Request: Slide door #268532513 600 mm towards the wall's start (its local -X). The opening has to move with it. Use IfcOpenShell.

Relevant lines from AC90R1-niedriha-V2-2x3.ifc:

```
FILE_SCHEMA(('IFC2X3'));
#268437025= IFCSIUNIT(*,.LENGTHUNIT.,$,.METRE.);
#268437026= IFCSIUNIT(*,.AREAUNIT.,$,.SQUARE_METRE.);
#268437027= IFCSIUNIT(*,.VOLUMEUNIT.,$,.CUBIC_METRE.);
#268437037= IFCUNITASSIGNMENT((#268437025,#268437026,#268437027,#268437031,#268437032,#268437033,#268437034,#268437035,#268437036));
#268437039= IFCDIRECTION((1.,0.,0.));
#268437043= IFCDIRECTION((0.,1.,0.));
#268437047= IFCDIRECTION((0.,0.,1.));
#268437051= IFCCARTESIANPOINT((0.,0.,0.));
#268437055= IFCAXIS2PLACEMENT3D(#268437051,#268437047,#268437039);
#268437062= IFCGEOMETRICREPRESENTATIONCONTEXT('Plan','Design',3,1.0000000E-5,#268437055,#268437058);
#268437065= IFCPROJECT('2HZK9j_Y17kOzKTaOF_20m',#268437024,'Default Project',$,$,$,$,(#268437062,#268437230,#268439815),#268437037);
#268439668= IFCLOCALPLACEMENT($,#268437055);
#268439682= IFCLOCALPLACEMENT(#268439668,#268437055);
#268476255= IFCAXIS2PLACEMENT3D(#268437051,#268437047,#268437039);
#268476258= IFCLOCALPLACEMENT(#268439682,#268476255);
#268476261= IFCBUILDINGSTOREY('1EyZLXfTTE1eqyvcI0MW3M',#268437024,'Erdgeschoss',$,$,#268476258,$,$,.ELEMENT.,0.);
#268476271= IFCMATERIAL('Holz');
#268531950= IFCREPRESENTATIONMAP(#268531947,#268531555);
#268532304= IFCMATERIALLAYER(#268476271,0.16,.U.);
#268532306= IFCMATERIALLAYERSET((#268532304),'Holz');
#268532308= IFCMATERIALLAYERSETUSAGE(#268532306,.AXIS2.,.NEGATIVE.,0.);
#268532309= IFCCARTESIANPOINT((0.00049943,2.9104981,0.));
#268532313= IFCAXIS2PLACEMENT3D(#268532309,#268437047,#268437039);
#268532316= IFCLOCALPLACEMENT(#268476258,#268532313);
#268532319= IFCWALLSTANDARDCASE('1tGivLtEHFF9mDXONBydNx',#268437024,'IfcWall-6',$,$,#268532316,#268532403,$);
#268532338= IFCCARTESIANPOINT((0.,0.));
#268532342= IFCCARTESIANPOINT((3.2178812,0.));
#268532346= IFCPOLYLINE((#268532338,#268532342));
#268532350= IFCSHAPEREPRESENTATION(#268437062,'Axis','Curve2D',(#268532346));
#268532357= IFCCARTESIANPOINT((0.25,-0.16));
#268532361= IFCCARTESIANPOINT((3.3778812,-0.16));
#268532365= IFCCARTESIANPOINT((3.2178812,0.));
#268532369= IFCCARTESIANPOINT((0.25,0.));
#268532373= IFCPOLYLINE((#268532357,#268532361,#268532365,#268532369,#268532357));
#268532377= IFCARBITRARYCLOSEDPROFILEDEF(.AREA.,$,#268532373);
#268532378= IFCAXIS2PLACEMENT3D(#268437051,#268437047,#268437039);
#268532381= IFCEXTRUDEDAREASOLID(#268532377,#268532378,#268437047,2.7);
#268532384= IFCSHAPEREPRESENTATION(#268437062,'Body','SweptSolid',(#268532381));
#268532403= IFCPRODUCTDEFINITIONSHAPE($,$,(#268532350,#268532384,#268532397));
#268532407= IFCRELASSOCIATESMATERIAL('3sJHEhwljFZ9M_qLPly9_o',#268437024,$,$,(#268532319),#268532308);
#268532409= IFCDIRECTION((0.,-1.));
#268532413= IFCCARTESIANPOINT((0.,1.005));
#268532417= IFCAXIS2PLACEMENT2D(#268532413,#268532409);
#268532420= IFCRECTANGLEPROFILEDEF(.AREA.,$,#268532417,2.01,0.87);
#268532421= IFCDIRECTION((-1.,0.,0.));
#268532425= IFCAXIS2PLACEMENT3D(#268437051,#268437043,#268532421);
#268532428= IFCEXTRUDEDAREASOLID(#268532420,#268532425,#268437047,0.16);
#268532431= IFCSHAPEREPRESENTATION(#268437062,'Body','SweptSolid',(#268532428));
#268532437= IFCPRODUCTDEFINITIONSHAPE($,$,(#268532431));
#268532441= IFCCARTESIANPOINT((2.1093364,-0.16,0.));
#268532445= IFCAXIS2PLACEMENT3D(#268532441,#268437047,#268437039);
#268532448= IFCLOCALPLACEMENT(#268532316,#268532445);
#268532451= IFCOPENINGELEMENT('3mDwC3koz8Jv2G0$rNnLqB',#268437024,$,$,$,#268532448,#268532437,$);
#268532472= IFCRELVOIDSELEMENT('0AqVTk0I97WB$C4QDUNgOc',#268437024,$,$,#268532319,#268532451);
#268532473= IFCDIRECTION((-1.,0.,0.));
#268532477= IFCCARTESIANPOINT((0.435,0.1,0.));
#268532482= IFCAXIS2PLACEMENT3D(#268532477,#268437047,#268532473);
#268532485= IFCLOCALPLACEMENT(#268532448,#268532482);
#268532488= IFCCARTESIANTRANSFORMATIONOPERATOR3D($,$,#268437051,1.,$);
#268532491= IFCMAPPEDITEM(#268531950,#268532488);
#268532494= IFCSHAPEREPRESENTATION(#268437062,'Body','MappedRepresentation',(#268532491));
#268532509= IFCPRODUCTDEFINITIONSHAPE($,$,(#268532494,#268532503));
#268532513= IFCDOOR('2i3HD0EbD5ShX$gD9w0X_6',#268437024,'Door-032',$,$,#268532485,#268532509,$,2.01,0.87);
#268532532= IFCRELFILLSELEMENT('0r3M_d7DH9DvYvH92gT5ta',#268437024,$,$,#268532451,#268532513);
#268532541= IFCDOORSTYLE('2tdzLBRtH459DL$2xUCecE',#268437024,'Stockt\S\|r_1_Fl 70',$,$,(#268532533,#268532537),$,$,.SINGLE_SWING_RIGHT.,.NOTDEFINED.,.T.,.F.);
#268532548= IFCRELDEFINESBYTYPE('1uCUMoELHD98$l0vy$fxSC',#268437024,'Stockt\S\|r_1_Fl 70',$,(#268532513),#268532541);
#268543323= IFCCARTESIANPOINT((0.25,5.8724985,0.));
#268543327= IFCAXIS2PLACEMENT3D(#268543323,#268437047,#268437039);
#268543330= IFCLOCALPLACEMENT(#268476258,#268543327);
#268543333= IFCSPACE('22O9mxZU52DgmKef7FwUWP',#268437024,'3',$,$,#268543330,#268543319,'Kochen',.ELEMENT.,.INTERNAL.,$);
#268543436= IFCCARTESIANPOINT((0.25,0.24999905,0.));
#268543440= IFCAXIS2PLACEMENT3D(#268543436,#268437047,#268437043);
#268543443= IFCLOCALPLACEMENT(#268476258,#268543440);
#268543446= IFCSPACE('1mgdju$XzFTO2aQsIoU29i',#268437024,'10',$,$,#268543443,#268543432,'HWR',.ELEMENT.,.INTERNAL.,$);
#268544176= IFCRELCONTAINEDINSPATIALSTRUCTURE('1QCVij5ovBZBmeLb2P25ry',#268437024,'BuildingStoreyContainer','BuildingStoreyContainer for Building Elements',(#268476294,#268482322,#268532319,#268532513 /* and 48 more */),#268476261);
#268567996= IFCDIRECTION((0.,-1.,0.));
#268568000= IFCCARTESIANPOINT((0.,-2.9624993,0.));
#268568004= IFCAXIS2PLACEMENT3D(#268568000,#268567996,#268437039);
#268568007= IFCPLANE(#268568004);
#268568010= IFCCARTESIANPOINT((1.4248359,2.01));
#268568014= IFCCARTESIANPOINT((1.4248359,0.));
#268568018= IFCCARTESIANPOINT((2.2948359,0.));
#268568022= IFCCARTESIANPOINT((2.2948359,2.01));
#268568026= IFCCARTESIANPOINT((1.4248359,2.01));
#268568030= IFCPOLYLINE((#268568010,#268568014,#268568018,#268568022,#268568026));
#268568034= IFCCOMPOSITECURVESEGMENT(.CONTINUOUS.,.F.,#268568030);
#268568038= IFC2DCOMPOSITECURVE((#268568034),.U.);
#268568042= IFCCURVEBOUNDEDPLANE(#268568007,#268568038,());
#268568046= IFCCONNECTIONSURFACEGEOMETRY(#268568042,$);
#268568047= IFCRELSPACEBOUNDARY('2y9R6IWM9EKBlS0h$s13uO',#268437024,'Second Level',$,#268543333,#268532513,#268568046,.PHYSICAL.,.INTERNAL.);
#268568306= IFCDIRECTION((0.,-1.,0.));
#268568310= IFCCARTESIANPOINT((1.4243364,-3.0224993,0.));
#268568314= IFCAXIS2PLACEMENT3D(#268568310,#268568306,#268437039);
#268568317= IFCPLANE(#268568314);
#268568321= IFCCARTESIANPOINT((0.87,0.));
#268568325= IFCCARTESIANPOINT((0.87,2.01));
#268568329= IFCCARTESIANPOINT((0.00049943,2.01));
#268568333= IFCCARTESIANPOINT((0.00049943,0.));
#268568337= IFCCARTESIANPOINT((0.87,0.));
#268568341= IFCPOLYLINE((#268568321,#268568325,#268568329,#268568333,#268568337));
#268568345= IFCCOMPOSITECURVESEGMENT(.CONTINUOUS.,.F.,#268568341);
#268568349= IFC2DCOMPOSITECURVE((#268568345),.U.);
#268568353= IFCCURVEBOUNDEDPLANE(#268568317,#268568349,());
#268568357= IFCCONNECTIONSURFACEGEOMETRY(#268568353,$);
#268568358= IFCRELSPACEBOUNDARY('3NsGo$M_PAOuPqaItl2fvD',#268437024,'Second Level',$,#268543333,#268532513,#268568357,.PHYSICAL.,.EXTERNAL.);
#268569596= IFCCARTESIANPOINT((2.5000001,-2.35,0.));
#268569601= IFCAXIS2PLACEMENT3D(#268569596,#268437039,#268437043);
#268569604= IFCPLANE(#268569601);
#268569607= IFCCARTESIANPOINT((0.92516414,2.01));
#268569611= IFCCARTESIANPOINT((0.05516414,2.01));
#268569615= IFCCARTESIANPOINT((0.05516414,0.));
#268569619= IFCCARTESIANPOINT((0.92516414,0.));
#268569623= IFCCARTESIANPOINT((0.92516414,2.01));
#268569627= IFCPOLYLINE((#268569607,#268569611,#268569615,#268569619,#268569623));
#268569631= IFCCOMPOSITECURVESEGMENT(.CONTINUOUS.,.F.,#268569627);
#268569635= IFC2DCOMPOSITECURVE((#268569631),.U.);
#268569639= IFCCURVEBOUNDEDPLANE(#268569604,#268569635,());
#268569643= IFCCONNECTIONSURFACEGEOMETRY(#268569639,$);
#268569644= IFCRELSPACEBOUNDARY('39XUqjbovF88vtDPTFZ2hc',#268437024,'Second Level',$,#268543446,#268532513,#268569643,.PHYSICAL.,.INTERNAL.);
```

```python
import numpy as np
import ifcopenshell
import ifcopenshell.api.geometry
import ifcopenshell.util.placement

model = ifcopenshell.open("AC90R1-niedriha-V2-2x3.ifc")

door = model.by_guid("2i3HD0EbD5ShX$gD9w0X_6")
opening = door.FillsVoids[0].RelatingOpeningElement
wall = opening.VoidsElements[0].RelatingBuildingElement

wall_matrix = ifcopenshell.util.placement.get_local_placement(wall.ObjectPlacement)
shift = wall_matrix[:3, 0] * -0.6
before = ifcopenshell.util.placement.get_local_placement(door.ObjectPlacement)[:3, 3].copy()

# The door is placed relative to its opening, so it follows when the opening moves.
matrix = ifcopenshell.util.placement.get_local_placement(opening.ObjectPlacement)
matrix[:3, 3] += shift
ifcopenshell.api.geometry.edit_object_placement(
    model, product=opening, matrix=matrix, is_si=False, should_transform_children=True
)

# Space boundary surfaces are stored in each space's coordinates; move them too.
for rel in door.ProvidesBoundaries:
    if not rel.ConnectionGeometry:
        continue
    surface = rel.ConnectionGeometry.SurfaceOnRelatingElement.BasisSurface
    space_matrix = ifcopenshell.util.placement.get_local_placement(rel.RelatingSpace.ObjectPlacement)
    point = np.array(surface.Position.Location.Coordinates) + space_matrix[:3, :3].T @ shift
    surface.Position = model.createIfcAxis2Placement3D(
        model.createIfcCartesianPoint(point.tolist()), surface.Position.Axis, surface.Position.RefDirection
    )

after = ifcopenshell.util.placement.get_local_placement(door.ObjectPlacement)[:3, 3]
print("door moved by", (after - before).round(3) + 0.0)

model.write("AC90R1-niedriha-V2-2x3-out.ifc")
```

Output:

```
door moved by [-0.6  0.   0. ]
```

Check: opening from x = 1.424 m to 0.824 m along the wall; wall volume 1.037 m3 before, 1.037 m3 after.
